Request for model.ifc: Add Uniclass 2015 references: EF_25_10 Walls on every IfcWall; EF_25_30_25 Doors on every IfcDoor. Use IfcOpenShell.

First a look at what the model holds.

```python
import ifcopenshell

model = ifcopenshell.open("model.ifc")
print(model.schema)
print("classifications:", [c.Name for c in model.by_type("IfcClassification")])
for ifc_class in ("IfcDoor", "IfcRoof", "IfcStair", "IfcWall", "IfcWindow"):
    print(ifc_class, len(model.by_type(ifc_class)))
```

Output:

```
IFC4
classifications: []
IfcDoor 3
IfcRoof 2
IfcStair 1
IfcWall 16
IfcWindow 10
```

```python
import ifcopenshell
import ifcopenshell.api.classification

model = ifcopenshell.open("model.ifc")

system = ifcopenshell.api.classification.add_classification(model, classification="Uniclass 2015")

codes = {
    "IfcWall": ("EF_25_10", "Walls"),
    "IfcDoor": ("EF_25_30_25", "Doors"),
}
for ifc_class, (code, name) in codes.items():
    products = model.by_type(ifc_class)
    ifcopenshell.api.classification.add_reference(
        model, products=products, classification=system, identification=code, name=name
    )
    print(code, len(products))

model.write("model_rev.ifc")
```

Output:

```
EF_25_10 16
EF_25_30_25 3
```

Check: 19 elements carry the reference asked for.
